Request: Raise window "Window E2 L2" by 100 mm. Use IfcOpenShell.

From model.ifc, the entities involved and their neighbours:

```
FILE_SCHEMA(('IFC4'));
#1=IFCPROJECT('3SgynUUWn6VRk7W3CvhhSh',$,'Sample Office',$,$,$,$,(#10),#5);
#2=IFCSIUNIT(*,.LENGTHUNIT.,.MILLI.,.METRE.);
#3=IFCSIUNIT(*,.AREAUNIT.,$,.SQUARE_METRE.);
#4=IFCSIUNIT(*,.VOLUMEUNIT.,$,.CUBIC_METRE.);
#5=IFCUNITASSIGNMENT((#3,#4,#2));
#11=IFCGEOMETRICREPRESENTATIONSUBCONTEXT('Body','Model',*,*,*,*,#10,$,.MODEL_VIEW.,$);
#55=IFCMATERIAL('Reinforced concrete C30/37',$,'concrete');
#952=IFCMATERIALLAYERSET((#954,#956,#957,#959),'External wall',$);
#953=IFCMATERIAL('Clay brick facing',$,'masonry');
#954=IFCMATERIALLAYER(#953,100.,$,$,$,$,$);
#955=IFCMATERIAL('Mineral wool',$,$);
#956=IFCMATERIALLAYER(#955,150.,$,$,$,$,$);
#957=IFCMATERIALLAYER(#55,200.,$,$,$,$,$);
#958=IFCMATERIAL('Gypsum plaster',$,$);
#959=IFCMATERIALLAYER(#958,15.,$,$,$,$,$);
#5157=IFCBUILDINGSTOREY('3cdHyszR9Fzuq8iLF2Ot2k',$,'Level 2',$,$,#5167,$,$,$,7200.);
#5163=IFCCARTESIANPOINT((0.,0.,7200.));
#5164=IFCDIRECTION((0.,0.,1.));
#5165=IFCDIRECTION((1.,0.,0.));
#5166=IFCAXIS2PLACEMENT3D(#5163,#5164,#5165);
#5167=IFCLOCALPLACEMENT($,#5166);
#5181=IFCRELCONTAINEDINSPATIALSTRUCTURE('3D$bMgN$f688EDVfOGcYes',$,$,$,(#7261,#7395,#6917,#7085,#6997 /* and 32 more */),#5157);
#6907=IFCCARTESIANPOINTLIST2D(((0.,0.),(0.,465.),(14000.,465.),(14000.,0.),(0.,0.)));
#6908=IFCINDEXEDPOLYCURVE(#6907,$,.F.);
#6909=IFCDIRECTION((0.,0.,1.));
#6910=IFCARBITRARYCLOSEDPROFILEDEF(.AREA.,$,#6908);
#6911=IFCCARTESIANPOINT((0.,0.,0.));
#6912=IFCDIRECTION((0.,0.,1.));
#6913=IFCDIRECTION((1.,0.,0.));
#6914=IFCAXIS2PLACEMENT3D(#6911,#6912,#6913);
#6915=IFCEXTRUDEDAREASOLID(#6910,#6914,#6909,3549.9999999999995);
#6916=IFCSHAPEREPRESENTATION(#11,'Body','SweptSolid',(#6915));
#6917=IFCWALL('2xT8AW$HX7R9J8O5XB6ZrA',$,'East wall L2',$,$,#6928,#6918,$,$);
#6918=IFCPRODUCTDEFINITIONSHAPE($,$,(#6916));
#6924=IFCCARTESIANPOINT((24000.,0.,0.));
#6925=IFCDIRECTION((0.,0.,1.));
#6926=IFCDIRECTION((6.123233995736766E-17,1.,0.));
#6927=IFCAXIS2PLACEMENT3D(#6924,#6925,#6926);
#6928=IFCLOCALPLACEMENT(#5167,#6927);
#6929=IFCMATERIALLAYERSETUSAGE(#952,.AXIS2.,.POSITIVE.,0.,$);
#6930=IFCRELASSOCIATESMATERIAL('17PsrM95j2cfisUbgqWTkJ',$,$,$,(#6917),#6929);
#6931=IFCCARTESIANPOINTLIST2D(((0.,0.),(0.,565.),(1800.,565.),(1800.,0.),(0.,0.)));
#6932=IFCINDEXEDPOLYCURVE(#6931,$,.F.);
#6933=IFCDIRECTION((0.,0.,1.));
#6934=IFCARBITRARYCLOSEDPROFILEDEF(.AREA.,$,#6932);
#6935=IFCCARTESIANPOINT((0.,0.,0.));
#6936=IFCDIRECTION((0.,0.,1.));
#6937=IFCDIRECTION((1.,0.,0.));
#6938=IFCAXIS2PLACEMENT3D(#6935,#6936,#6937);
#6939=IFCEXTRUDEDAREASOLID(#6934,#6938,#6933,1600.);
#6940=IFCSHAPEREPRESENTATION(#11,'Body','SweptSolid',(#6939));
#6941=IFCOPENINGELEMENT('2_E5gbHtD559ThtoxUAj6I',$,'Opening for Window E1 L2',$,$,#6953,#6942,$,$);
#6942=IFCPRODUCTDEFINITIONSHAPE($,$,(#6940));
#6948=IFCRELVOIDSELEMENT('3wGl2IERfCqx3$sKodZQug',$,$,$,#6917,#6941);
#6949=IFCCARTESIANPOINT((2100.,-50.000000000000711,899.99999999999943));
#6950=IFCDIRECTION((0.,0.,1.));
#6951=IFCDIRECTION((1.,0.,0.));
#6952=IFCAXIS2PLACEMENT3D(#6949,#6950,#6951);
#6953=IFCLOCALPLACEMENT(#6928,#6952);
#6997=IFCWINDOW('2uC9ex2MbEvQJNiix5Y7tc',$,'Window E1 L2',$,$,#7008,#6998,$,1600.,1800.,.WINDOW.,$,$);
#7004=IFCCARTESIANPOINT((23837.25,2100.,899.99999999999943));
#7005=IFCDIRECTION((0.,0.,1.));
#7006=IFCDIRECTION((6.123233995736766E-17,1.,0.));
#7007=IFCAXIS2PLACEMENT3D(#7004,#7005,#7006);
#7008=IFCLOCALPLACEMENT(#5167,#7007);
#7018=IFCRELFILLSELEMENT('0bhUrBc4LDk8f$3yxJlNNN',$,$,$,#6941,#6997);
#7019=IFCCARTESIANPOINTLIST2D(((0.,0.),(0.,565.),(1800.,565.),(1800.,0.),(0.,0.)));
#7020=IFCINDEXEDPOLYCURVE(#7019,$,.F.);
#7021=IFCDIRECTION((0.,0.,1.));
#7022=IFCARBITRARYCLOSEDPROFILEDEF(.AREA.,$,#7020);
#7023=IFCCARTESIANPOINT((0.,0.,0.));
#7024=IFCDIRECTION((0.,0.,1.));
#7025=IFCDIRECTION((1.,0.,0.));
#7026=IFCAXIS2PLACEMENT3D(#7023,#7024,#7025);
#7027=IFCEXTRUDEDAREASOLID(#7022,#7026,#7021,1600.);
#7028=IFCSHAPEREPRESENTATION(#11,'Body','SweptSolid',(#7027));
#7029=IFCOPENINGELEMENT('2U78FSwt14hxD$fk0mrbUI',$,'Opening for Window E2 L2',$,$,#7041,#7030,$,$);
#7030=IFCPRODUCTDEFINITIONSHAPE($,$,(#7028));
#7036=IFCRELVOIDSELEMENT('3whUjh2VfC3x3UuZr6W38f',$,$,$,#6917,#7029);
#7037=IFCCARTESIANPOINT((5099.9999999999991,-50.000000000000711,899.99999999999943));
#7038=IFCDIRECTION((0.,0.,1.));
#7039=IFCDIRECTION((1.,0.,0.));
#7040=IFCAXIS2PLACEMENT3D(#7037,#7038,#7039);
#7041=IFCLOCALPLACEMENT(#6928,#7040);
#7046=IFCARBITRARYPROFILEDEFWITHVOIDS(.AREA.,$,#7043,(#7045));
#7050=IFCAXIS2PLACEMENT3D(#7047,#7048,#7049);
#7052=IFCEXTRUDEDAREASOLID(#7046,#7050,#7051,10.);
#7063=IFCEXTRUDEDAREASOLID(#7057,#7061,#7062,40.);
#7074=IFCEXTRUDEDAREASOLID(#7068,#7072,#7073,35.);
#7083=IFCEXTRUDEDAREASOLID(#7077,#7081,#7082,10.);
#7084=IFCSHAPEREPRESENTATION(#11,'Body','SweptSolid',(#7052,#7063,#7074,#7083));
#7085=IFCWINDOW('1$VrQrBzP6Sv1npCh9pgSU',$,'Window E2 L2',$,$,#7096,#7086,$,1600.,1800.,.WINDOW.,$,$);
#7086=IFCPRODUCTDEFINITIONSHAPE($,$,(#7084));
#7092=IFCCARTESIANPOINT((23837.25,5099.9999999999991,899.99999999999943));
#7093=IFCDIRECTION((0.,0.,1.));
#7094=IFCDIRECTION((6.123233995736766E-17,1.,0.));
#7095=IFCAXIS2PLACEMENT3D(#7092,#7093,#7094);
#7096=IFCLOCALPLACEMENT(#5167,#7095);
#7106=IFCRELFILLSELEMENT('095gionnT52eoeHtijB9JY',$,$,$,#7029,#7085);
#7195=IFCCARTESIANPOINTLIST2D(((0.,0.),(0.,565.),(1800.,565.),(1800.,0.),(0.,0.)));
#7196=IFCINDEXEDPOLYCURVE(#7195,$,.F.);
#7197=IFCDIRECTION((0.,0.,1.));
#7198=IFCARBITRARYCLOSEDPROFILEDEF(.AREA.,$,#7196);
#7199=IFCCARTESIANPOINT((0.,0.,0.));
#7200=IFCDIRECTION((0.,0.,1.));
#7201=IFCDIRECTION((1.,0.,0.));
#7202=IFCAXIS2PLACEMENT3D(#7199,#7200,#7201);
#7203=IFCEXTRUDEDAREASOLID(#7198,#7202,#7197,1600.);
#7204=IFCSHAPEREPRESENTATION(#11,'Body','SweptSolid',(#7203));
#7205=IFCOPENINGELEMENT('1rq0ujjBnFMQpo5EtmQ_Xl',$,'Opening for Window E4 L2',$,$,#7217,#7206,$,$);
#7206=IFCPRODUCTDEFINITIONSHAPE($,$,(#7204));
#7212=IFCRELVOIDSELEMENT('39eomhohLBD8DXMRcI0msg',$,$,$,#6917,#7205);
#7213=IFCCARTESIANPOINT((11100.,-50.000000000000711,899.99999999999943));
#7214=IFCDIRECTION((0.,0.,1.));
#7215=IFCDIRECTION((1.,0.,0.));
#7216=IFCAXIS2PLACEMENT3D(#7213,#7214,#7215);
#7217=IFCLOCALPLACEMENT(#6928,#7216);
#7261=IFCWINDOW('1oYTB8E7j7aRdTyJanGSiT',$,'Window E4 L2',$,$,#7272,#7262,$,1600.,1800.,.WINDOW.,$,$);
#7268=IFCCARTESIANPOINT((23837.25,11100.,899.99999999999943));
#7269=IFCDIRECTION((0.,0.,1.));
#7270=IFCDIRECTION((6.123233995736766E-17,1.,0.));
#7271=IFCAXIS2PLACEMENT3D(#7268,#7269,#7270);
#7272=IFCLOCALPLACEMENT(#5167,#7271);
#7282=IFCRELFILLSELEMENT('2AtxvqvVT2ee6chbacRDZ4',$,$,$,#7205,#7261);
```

```python
import numpy as np
import ifcopenshell
import ifcopenshell.api.geometry
import ifcopenshell.util.placement
import ifcopenshell.util.unit

model = ifcopenshell.open("model.ifc")
unit_scale = ifcopenshell.util.unit.calculate_unit_scale(model)

window = model.by_id(7085)
opening = window.FillsVoids[0].RelatingOpeningElement
dz = 100.0

shift = np.array([0.0, 0.0, dz])
# The window is not placed relative to its opening, so move both.
for product in (opening, window):
    matrix = ifcopenshell.util.placement.get_local_placement(product.ObjectPlacement)
    matrix[:3, 3] += shift
    ifcopenshell.api.geometry.edit_object_placement(model, product=product, matrix=matrix, is_si=False)

print(f"moved by {dz * unit_scale:+.3f} m")

model.write("model_updated.ifc")
```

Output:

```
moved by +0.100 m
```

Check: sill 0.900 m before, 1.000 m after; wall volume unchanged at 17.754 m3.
